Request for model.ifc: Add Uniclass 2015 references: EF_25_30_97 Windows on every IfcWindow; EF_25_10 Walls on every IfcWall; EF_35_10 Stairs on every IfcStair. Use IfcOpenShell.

First a look at what the model holds.

```python
import ifcopenshell

model = ifcopenshell.open("model.ifc")
print(model.schema)
print("classifications:", [c.Name for c in model.by_type("IfcClassification")])
for ifc_class in ("IfcDoor", "IfcRoof", "IfcStair", "IfcWall", "IfcWindow"):
    print(ifc_class, len(model.by_type(ifc_class)))
```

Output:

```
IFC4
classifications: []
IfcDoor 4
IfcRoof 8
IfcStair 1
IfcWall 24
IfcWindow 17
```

```python
import ifcopenshell
import ifcopenshell.api.classification

model = ifcopenshell.open("model.ifc")

system = ifcopenshell.api.classification.add_classification(model, classification="Uniclass 2015")

codes = {
    "IfcWindow": ("EF_25_30_97", "Windows"),
    "IfcWall": ("EF_25_10", "Walls"),
    "IfcStair": ("EF_35_10", "Stairs"),
}
for ifc_class, (code, name) in codes.items():
    products = model.by_type(ifc_class)
    ifcopenshell.api.classification.add_reference(
        model, products=products, classification=system, identification=code, name=name
    )
    print(code, len(products))

model.write("model_updated.ifc")
```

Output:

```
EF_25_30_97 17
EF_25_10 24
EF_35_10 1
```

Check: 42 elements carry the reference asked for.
